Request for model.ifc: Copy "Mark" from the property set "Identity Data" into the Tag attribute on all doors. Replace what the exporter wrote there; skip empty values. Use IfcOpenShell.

First a look at what the model holds.

```python
import ifcopenshell
import ifcopenshell.util.element

model = ifcopenshell.open("model.ifc")
print(model.schema)
doors = model.by_type("IfcDoor")
print(len(doors), "doors")
for e in doors[:8]:
    source = ifcopenshell.util.element.get_pset(e, "Identity Data", "Mark")
    target = e.Tag
    print(e.id(), repr(source), repr(target), sep=" | ")
```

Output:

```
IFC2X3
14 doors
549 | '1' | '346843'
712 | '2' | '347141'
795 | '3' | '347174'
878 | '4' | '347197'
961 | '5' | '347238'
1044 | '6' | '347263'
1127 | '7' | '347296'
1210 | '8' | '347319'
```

```python
import ifcopenshell
import ifcopenshell.util.element

model = ifcopenshell.open("model.ifc")

count = 0
for e in model.by_type("IfcDoor"):
    value = ifcopenshell.util.element.get_pset(e, "Identity Data", "Mark")
    current = e.Tag
    if not value or not value.strip() or current == value:
        continue
    e.Tag = value
    count += 1

print(count, "doors updated")

model.write("model_edited.ifc")
```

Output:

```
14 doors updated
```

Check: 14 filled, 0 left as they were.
